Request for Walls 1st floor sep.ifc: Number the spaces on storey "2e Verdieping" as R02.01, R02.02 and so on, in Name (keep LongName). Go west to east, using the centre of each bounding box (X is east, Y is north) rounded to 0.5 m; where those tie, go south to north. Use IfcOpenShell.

First a look at what the model holds.

```python
import ifcopenshell
import ifcopenshell.util.element
import ifcopenshell.util.placement

model = ifcopenshell.open("Walls 1st floor sep.ifc")
print(model.schema)
storey = next(s for s in model.by_type("IfcBuildingStorey") if s.Name == "2e Verdieping")
spaces = [e for e in ifcopenshell.util.element.get_decomposition(storey) if e.is_a("IfcSpace")]
for e in sorted(spaces, key=lambda e: e.id()):
    origin = ifcopenshell.util.placement.get_local_placement(e.ObjectPlacement)[:3, 3]
    print(e.id(), e.Name, e.LongName, origin.round(2) + 0.0, sep=" | ")
```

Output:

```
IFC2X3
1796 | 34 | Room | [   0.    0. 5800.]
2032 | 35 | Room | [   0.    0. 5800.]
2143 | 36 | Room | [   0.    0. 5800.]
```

```python
import ifcopenshell
import ifcopenshell.geom
import ifcopenshell.util.element
import ifcopenshell.util.shape

model = ifcopenshell.open("Walls 1st floor sep.ifc")
settings = ifcopenshell.geom.settings()
settings.set("use-world-coords", True)


def centre(element):
    shape = ifcopenshell.geom.create_shape(settings, element)
    return ifcopenshell.util.shape.get_bbox_centroid(shape.geometry)


storey = next(s for s in model.by_type("IfcBuildingStorey") if s.Name == "2e Verdieping")
spaces = [e for e in ifcopenshell.util.element.get_decomposition(storey) if e.is_a("IfcSpace")]

# Insertion points can sit at a corner or the storey origin, so sort by the geometry (in metres).
centres = {e: centre(e) for e in spaces}
spaces.sort(key=lambda e: (round(centres[e][0] / 0.5), centres[e][1]))

for i, e in enumerate(spaces, start=1):
    number = f"R02.{i:02d}"
    e.Name = number
    print(e.id(), number)

model.write("Walls 1st floor sep-out.ifc")
```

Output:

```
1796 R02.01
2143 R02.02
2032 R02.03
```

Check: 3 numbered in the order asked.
